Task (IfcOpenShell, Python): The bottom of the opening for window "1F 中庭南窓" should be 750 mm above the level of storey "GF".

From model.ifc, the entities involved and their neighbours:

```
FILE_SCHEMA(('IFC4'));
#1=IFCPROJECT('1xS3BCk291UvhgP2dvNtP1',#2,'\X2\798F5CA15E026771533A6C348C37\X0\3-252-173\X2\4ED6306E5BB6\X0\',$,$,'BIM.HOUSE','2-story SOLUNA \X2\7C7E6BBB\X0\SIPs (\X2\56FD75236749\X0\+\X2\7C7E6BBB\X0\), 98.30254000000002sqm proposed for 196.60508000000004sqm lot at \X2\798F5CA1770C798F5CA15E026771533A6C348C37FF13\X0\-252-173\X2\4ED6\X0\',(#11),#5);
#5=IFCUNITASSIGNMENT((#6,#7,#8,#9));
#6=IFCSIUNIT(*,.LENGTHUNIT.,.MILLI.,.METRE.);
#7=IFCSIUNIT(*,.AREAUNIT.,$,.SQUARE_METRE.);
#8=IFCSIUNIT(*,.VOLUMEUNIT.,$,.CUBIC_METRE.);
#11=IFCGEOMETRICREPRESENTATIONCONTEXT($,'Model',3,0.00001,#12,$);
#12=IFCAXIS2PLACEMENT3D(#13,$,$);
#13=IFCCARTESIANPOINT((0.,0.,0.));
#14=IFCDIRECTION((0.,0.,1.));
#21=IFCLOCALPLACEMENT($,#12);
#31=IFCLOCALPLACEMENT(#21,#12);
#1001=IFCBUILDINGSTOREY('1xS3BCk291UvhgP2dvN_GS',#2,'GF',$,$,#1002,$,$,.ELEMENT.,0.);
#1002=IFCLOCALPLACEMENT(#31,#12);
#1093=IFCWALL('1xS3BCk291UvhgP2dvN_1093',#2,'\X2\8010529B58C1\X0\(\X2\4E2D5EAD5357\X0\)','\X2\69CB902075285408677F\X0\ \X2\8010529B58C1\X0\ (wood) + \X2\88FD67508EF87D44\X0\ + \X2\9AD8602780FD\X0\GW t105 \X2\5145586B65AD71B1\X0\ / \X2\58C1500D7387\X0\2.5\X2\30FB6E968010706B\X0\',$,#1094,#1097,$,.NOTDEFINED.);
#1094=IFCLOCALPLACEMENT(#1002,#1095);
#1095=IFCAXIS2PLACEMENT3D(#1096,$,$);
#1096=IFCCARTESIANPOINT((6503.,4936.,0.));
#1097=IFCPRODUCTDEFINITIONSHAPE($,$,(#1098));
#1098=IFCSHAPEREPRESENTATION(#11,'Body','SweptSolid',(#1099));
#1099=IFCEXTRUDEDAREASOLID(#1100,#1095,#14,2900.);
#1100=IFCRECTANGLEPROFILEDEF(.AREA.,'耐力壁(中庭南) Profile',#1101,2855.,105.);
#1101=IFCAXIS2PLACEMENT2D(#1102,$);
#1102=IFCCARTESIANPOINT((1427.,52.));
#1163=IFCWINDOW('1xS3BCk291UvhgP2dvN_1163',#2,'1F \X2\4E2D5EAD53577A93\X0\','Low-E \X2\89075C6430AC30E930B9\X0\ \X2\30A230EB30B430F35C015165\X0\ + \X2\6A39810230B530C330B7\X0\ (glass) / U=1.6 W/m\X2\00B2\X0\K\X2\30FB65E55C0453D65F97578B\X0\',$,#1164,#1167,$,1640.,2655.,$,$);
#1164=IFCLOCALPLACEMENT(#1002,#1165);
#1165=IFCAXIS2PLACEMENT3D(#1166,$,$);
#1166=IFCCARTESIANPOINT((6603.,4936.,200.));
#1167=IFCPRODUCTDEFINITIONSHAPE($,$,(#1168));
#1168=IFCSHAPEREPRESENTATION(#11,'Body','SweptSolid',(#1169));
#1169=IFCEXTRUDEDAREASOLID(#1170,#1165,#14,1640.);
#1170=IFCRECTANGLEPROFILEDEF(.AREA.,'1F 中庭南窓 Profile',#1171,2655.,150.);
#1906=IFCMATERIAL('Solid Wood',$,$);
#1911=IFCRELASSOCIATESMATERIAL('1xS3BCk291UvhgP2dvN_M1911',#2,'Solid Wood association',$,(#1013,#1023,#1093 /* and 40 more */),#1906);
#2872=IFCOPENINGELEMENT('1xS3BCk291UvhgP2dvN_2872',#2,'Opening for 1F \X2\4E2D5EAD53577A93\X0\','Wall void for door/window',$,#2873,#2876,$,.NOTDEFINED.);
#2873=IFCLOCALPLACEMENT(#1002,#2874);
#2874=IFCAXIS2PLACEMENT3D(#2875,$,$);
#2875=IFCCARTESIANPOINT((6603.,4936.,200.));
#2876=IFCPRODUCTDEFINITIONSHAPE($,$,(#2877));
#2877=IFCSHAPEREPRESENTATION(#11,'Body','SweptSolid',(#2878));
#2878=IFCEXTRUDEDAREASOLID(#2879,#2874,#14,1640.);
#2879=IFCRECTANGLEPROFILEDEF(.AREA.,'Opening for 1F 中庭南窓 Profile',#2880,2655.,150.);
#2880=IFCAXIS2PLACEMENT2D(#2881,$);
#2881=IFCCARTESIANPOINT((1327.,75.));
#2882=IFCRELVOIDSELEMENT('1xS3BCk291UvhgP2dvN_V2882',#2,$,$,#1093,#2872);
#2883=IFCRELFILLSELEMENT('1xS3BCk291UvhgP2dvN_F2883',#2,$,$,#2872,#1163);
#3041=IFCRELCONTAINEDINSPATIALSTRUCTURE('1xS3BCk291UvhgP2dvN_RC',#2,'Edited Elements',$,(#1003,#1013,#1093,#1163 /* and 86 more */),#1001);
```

```python
import numpy as np
import ifcopenshell
import ifcopenshell.api.geometry
import ifcopenshell.geom
import ifcopenshell.util.element
import ifcopenshell.util.placement
import ifcopenshell.util.shape
import ifcopenshell.util.unit

model = ifcopenshell.open("model.ifc")
unit_scale = ifcopenshell.util.unit.calculate_unit_scale(model)

window = model.by_guid("1xS3BCk291UvhgP2dvN_1163")
opening = window.FillsVoids[0].RelatingOpeningElement
storey = ifcopenshell.util.element.get_container(window, ifc_class="IfcBuildingStorey")
level = ifcopenshell.util.placement.get_local_placement(storey.ObjectPlacement)[2, 3]

# The opening's origin need not be at the sill, so measure its lowest point.
shape = ifcopenshell.geom.create_shape(ifcopenshell.geom.settings(), opening)
bottom = ifcopenshell.util.shape.get_shape_bottom_elevation(shape, shape.geometry) / unit_scale
dz = level + 0.75 / unit_scale - bottom

shift = np.array([0.0, 0.0, dz])
# The window is not placed relative to its opening, so move both.
for product in (opening, window):
    matrix = ifcopenshell.util.placement.get_local_placement(product.ObjectPlacement)
    matrix[:3, 3] += shift
    ifcopenshell.api.geometry.edit_object_placement(model, product=product, matrix=matrix, is_si=False)

print(f"moved by {dz * unit_scale:+.3f} m")

model.write("model_edited.ifc")
```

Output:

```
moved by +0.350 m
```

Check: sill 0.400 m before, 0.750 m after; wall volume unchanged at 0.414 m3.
